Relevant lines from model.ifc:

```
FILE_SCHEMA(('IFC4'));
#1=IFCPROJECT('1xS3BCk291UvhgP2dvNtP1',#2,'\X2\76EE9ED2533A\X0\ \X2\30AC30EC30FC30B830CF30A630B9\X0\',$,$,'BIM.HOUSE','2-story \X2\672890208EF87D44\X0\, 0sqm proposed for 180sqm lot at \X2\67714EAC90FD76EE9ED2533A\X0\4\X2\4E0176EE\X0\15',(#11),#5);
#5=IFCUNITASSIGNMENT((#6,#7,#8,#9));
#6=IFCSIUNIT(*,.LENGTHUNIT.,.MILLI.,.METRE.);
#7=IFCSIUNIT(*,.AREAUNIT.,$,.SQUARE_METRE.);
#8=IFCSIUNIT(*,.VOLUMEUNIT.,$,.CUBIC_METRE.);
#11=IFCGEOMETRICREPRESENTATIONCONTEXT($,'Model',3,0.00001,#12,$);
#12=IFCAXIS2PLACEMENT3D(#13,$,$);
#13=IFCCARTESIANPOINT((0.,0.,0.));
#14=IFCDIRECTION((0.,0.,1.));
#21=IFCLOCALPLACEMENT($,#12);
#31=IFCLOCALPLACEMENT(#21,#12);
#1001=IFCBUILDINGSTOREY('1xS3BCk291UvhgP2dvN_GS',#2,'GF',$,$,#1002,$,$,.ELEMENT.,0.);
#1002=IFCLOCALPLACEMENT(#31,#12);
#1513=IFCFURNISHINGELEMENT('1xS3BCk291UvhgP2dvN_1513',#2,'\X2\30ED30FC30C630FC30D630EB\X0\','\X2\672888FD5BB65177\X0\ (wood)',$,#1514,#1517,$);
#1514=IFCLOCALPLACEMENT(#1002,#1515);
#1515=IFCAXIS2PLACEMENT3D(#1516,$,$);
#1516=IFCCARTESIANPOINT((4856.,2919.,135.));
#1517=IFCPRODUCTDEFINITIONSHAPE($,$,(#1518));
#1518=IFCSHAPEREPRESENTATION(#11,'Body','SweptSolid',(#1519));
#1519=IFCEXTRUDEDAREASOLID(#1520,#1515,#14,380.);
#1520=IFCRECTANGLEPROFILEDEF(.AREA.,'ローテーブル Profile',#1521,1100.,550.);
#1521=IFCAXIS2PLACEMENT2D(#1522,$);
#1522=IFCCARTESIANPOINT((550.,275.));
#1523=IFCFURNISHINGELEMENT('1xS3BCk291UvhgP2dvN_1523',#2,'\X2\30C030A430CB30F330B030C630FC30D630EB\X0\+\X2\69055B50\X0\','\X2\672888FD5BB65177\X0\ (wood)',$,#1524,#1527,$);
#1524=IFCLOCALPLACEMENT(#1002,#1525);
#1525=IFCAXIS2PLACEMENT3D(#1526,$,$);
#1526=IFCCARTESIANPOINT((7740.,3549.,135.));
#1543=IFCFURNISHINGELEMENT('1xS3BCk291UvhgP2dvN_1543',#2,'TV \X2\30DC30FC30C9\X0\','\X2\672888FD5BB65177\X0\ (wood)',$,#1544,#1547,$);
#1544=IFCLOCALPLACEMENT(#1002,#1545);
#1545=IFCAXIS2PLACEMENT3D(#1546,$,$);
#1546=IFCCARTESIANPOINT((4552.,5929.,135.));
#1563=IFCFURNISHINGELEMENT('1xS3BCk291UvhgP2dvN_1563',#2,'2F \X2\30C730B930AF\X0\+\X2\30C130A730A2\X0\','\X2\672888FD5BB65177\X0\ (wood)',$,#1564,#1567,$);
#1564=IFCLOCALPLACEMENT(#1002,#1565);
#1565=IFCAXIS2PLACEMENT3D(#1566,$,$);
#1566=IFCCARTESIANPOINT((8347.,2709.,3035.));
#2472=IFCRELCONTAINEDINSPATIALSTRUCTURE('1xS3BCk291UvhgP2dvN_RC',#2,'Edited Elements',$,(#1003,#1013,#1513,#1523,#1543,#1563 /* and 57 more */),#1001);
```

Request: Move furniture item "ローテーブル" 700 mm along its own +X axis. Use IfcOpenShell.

```python
import ifcopenshell
import ifcopenshell.api.geometry
import ifcopenshell.util.placement
import ifcopenshell.util.unit

model = ifcopenshell.open("model.ifc")
unit_scale = ifcopenshell.util.unit.calculate_unit_scale(model)

item = model.by_guid("1xS3BCk291UvhgP2dvN_1513")
matrix = ifcopenshell.util.placement.get_local_placement(item.ObjectPlacement)
matrix[:3, 3] += matrix[:3, 0] * 0.7 / unit_scale
ifcopenshell.api.geometry.edit_object_placement(model, product=item, matrix=matrix, is_si=False)

print(ifcopenshell.util.placement.get_local_placement(item.ObjectPlacement).round(3) + 0.0)

model.write("model-out.ifc")
```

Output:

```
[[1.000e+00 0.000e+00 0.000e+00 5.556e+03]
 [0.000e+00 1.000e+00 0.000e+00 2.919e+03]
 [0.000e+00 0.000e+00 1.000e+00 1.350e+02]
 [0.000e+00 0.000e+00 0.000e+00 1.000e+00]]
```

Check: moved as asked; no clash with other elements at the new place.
